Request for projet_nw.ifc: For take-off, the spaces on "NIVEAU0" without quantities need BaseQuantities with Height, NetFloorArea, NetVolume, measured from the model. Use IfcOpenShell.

First a look at what the model holds.

```python
import ifcopenshell
import ifcopenshell.util.element
import ifcopenshell.util.unit

model = ifcopenshell.open("projet_nw.ifc")
print(model.schema)
for unit_type in ("LENGTHUNIT", "AREAUNIT", "VOLUMEUNIT"):
    print(unit_type, ifcopenshell.util.unit.calculate_unit_scale(model, unit_type))
storey = next(s for s in model.by_type("IfcBuildingStorey") if s.Name == "NIVEAU0")
spaces = [e for e in ifcopenshell.util.element.get_decomposition(storey) if e.is_a("IfcSpace")]
for e in sorted(spaces, key=lambda e: e.id()):
    print(e.id(), e.is_a(), e.Name, list(ifcopenshell.util.element.get_psets(e, qtos_only=True)), sep=" | ")
```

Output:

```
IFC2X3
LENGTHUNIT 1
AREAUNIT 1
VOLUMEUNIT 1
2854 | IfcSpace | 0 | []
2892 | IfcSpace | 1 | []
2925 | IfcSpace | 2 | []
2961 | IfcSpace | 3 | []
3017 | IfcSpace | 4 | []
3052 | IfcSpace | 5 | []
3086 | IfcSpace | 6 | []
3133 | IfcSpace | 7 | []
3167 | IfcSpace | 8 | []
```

```python
import ifcopenshell
import ifcopenshell.api.pset
import ifcopenshell.geom
import ifcopenshell.util.element
import ifcopenshell.util.shape
import ifcopenshell.util.unit

model = ifcopenshell.open("projet_nw.ifc")
unit_scale = ifcopenshell.util.unit.calculate_unit_scale(model)
area_scale = ifcopenshell.util.unit.calculate_unit_scale(model, "AREAUNIT")
volume_scale = ifcopenshell.util.unit.calculate_unit_scale(model, "VOLUMEUNIT")
settings = ifcopenshell.geom.settings()

storey = next(s for s in model.by_type("IfcBuildingStorey") if s.Name == "NIVEAU0")
spaces = [e for e in ifcopenshell.util.element.get_decomposition(storey) if e.is_a("IfcSpace")]

for e in sorted(spaces, key=lambda e: e.id()):
    if ifcopenshell.util.element.get_psets(e, qtos_only=True, should_inherit=False):
        continue
    # Geometry comes back in metres, in the element's own axes.
    shape = ifcopenshell.geom.create_shape(settings, e)
    values = {
        "Height": ifcopenshell.util.shape.get_z(shape.geometry) / unit_scale,
        "NetFloorArea": ifcopenshell.util.shape.get_footprint_area(shape.geometry) / area_scale,
        "NetVolume": ifcopenshell.util.shape.get_volume(shape.geometry) / volume_scale,
    }
    qto = ifcopenshell.api.pset.add_qto(model, product=e, name="BaseQuantities")
    ifcopenshell.api.pset.edit_qto(model, qto=qto, properties=values)
    print(e.id(), {k: round(v, 3) for k, v in values.items()})

model.write("projet_nw_v2.ifc")
```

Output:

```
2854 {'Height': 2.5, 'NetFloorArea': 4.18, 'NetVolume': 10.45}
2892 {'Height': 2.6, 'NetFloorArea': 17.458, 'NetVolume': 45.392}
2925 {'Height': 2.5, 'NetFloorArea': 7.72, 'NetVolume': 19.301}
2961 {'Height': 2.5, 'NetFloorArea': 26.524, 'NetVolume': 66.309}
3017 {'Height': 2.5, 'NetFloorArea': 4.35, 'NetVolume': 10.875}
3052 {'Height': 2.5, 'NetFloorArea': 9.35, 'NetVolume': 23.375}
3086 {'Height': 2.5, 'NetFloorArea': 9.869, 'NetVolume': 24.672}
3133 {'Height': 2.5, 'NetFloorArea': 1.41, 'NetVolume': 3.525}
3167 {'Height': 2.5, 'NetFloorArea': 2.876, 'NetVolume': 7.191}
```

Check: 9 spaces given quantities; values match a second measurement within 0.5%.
